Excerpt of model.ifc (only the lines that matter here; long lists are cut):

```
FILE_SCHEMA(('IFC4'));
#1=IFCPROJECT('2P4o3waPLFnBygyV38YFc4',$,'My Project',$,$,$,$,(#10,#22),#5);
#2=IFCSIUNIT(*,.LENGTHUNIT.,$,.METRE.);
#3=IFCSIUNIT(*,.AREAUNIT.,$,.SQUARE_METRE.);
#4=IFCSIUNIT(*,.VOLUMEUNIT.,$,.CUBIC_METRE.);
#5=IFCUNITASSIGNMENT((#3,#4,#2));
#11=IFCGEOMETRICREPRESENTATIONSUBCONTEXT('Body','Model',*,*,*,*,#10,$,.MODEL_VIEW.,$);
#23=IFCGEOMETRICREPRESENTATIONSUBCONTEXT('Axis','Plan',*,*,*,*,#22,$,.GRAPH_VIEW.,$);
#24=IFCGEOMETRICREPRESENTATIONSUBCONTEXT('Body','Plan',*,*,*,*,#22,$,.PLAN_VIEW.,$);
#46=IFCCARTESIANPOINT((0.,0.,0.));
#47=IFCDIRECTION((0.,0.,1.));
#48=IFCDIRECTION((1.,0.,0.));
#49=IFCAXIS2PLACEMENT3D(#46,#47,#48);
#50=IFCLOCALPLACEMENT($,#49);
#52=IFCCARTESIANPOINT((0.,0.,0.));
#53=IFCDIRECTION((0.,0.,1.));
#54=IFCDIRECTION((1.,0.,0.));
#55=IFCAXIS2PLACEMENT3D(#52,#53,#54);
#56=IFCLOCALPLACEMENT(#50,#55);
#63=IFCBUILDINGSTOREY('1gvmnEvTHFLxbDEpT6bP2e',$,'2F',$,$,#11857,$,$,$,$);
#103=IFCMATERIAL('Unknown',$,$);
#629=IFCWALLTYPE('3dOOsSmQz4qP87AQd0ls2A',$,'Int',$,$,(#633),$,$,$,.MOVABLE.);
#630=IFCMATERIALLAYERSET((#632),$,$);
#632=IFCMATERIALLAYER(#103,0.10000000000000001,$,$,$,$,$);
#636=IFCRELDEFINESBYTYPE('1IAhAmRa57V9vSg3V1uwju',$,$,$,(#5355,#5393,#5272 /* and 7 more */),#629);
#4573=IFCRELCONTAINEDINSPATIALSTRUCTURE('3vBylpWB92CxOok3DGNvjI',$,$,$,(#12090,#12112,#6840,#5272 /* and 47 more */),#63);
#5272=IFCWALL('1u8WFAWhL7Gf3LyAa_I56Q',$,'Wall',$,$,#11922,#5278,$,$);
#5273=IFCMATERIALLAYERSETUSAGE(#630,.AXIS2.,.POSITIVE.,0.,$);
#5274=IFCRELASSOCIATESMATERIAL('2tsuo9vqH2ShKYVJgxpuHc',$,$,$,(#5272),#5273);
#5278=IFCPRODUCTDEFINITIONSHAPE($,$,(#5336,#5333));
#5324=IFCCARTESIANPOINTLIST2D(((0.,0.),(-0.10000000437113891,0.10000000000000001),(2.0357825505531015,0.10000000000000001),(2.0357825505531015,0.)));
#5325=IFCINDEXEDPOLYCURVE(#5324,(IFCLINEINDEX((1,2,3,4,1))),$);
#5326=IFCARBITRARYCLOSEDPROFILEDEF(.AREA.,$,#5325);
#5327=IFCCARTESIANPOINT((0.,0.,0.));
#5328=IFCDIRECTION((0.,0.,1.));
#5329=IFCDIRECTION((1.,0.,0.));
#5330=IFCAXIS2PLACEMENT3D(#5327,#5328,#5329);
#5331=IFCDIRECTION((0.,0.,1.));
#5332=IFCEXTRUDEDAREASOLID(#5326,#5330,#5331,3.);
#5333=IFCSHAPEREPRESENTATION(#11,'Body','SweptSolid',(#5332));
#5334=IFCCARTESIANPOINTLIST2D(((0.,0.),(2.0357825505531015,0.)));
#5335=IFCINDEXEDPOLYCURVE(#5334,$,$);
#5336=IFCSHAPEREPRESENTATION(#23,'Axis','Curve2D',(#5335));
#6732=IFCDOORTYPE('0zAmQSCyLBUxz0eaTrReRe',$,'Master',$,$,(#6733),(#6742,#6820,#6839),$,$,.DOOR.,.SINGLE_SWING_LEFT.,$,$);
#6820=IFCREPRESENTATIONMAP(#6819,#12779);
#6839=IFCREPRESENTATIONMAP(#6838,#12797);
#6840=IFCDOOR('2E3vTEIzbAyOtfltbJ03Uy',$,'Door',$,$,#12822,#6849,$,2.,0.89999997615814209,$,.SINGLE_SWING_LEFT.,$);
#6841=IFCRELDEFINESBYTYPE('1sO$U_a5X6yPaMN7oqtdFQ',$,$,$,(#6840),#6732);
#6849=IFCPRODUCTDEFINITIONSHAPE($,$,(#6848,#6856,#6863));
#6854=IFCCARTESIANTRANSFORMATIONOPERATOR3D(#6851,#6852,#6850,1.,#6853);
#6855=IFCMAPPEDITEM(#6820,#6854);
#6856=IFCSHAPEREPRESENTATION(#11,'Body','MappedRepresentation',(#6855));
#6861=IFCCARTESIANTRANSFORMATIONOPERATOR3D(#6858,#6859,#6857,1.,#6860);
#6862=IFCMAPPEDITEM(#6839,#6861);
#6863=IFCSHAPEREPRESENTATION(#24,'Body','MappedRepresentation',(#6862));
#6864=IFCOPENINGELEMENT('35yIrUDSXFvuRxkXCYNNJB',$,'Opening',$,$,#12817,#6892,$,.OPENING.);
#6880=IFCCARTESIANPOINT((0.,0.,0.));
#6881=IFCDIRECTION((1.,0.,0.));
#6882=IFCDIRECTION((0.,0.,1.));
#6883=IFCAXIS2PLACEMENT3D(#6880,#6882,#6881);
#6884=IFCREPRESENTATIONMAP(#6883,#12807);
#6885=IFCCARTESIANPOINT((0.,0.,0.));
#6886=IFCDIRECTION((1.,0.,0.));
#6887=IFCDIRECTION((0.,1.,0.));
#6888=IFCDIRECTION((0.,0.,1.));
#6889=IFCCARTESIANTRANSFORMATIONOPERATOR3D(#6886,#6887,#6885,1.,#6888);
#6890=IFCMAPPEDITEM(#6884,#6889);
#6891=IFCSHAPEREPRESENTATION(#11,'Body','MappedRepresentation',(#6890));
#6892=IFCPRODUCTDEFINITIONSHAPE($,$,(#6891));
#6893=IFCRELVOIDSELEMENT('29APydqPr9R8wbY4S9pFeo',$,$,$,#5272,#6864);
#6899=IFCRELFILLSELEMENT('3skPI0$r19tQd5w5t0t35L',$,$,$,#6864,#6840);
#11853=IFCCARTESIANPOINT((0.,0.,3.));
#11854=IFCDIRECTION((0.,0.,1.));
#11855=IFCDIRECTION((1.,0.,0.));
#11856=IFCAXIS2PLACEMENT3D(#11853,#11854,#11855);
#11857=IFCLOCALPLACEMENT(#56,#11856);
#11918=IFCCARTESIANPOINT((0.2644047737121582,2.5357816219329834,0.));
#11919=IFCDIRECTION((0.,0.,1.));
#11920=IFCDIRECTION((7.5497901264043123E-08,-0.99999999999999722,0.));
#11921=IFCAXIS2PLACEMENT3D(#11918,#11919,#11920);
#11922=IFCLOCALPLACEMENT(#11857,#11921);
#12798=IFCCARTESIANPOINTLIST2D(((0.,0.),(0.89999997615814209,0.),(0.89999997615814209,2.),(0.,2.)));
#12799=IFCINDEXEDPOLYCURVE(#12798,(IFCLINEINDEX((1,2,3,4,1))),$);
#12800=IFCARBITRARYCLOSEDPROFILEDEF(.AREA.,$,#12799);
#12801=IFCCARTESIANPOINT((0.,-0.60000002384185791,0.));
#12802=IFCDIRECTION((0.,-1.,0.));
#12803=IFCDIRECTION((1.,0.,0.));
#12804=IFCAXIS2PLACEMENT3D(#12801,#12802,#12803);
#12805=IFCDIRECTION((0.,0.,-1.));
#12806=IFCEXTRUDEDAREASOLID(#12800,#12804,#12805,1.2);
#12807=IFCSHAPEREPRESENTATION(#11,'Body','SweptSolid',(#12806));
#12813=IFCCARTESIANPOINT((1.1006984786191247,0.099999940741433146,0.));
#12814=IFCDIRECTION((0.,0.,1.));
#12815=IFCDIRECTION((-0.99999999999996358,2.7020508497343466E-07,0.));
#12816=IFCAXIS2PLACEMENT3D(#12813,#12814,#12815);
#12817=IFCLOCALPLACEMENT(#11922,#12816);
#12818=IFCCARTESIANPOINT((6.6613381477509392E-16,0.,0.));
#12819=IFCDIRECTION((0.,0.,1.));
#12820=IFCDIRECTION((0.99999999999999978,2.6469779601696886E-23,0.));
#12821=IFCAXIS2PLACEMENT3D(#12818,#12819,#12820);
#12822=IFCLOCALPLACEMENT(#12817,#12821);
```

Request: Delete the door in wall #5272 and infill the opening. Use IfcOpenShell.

```python
import ifcopenshell
import ifcopenshell.api.feature
import ifcopenshell.api.root
import ifcopenshell.geom
import ifcopenshell.util.shape

model = ifcopenshell.open("model.ifc")
settings = ifcopenshell.geom.settings()


def volume(element):
    """Net volume in cubic metres, openings subtracted."""
    shape = ifcopenshell.geom.create_shape(settings, element)
    return ifcopenshell.util.shape.get_volume(shape.geometry)


door = model.by_id(6840)
opening = door.FillsVoids[0].RelatingOpeningElement
wall = opening.VoidsElements[0].RelatingBuildingElement
before = volume(wall)

ifcopenshell.api.root.remove_product(model, product=door)
ifcopenshell.api.feature.remove_feature(model, feature=opening)

after = volume(wall)

print(f"wall volume {before:.3f} -> {after:.3f} m3")

model.write("model_updated.ifc")
```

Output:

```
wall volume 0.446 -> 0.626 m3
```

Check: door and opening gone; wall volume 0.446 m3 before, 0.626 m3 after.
